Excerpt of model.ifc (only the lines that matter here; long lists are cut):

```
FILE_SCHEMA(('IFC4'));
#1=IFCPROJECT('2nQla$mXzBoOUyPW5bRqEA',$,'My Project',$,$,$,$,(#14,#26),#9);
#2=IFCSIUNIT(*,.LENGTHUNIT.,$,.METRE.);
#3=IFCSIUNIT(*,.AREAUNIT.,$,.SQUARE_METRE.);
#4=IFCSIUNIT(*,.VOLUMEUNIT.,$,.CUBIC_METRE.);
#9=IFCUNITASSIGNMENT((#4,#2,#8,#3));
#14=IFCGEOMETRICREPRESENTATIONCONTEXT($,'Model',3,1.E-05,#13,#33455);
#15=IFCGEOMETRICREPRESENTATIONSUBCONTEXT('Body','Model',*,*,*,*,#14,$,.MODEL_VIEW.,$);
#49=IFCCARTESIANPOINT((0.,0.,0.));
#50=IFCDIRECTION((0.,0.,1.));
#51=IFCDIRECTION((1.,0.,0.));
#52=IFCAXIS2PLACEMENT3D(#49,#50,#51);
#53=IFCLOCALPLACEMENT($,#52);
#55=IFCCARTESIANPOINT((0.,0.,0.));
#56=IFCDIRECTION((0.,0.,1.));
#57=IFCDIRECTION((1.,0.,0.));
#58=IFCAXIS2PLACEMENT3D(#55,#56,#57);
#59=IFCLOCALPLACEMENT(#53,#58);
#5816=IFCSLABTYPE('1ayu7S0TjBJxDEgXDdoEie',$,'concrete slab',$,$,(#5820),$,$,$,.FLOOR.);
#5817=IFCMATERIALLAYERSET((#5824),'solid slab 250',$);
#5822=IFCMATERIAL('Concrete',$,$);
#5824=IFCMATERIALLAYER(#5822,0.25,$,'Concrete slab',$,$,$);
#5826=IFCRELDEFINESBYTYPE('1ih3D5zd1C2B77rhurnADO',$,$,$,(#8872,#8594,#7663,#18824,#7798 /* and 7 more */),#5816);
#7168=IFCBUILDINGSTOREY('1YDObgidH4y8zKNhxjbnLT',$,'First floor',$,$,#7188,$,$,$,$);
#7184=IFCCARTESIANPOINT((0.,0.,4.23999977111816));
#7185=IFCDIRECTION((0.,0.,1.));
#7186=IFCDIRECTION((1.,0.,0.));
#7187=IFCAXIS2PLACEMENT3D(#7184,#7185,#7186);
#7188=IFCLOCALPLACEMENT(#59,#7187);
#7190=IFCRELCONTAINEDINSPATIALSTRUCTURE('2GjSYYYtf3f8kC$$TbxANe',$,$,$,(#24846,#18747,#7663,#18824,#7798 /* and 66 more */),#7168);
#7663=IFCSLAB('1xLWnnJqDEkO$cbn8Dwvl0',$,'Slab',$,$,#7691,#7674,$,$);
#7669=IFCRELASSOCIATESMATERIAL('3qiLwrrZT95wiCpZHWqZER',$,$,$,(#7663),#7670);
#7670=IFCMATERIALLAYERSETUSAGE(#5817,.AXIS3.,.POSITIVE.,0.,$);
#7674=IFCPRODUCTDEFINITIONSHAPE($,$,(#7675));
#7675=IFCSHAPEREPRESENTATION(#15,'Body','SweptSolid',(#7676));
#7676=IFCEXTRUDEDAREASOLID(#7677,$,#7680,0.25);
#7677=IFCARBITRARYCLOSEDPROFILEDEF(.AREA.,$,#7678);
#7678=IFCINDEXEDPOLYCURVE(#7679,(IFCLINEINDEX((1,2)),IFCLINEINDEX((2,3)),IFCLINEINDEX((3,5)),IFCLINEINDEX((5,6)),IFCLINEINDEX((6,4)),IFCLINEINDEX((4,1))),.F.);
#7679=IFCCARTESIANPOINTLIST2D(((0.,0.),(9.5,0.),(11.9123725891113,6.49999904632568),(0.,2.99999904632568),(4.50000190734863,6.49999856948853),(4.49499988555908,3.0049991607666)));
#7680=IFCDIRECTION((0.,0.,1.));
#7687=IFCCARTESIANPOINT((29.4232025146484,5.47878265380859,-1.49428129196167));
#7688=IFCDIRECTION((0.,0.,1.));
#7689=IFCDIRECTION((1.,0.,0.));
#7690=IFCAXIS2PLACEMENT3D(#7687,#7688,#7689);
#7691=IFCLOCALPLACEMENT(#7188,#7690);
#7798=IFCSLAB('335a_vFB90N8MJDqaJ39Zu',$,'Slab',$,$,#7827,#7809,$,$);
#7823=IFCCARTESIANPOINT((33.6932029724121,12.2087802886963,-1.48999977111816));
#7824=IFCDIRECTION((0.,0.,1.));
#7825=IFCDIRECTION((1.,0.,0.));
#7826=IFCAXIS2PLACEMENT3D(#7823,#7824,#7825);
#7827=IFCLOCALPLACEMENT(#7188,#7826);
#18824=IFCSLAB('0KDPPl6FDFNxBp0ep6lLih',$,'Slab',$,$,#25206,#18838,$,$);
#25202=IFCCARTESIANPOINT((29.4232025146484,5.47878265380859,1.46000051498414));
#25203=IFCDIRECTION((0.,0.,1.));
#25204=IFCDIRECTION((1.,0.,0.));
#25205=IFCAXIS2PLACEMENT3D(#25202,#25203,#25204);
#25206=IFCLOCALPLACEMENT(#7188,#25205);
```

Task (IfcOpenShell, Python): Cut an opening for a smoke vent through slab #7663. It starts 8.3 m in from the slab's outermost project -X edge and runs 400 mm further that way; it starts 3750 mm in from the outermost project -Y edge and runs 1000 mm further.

```python
import numpy as np
import ifcopenshell
import ifcopenshell.api.feature
import ifcopenshell.api.geometry
import ifcopenshell.api.root
import ifcopenshell.geom
import ifcopenshell.util.placement
import ifcopenshell.util.representation
import ifcopenshell.util.shape
import ifcopenshell.util.unit

model = ifcopenshell.open("model.ifc")
unit_scale = ifcopenshell.util.unit.calculate_unit_scale(model)
settings = ifcopenshell.geom.settings()


def volume(element):
    """Net volume in cubic metres, openings subtracted."""
    shape = ifcopenshell.geom.create_shape(settings, element)
    return ifcopenshell.util.shape.get_volume(shape.geometry)


slab = model.by_guid("1xLWnnJqDEkO$cbn8Dwvl0")
before = volume(slab)

# Extent in the slab's own axes, in metres. The edges named are its -X and -Y sides.
slab_shape = ifcopenshell.geom.create_shape(settings, slab)
vertices = ifcopenshell.util.shape.get_vertices(slab_shape.geometry)
x_min, y_min, bottom = vertices.min(axis=0)
top = vertices[:, 2].max()

opening = ifcopenshell.api.root.create_entity(model, ifc_class="IfcOpeningElement", name="Smoke vent opening", predefined_type="OPENING")
context = ifcopenshell.util.representation.get_context(model, "Model", "Body", "MODEL_VIEW")
width, depth = 0.4, 1
outline = [(0.0, 0.0), (width, 0.0), (width, depth), (0.0, depth), (0.0, 0.0)]
# Overshoot both faces by 50 mm so the cut is clean.
shape = ifcopenshell.api.geometry.add_slab_representation(
    model, context=context, depth=top - bottom + 0.1, polyline=outline
)
ifcopenshell.api.geometry.assign_representation(model, product=opening, representation=shape)

matrix = ifcopenshell.util.placement.get_local_placement(slab.ObjectPlacement)
matrix[:, 3] = matrix @ np.append(np.array([x_min + 8.3, y_min + 3.75, bottom - 0.05]) / unit_scale, 1.0)
ifcopenshell.api.geometry.edit_object_placement(model, product=opening, matrix=matrix, is_si=False)
ifcopenshell.api.feature.add_feature(model, feature=opening, element=slab)

after = volume(slab)

print(f"slab volume {before:.3f} -> {after:.3f} m3")

model.write("model_updated.ifc")
```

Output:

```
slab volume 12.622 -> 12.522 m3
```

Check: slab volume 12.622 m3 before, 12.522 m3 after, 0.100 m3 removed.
